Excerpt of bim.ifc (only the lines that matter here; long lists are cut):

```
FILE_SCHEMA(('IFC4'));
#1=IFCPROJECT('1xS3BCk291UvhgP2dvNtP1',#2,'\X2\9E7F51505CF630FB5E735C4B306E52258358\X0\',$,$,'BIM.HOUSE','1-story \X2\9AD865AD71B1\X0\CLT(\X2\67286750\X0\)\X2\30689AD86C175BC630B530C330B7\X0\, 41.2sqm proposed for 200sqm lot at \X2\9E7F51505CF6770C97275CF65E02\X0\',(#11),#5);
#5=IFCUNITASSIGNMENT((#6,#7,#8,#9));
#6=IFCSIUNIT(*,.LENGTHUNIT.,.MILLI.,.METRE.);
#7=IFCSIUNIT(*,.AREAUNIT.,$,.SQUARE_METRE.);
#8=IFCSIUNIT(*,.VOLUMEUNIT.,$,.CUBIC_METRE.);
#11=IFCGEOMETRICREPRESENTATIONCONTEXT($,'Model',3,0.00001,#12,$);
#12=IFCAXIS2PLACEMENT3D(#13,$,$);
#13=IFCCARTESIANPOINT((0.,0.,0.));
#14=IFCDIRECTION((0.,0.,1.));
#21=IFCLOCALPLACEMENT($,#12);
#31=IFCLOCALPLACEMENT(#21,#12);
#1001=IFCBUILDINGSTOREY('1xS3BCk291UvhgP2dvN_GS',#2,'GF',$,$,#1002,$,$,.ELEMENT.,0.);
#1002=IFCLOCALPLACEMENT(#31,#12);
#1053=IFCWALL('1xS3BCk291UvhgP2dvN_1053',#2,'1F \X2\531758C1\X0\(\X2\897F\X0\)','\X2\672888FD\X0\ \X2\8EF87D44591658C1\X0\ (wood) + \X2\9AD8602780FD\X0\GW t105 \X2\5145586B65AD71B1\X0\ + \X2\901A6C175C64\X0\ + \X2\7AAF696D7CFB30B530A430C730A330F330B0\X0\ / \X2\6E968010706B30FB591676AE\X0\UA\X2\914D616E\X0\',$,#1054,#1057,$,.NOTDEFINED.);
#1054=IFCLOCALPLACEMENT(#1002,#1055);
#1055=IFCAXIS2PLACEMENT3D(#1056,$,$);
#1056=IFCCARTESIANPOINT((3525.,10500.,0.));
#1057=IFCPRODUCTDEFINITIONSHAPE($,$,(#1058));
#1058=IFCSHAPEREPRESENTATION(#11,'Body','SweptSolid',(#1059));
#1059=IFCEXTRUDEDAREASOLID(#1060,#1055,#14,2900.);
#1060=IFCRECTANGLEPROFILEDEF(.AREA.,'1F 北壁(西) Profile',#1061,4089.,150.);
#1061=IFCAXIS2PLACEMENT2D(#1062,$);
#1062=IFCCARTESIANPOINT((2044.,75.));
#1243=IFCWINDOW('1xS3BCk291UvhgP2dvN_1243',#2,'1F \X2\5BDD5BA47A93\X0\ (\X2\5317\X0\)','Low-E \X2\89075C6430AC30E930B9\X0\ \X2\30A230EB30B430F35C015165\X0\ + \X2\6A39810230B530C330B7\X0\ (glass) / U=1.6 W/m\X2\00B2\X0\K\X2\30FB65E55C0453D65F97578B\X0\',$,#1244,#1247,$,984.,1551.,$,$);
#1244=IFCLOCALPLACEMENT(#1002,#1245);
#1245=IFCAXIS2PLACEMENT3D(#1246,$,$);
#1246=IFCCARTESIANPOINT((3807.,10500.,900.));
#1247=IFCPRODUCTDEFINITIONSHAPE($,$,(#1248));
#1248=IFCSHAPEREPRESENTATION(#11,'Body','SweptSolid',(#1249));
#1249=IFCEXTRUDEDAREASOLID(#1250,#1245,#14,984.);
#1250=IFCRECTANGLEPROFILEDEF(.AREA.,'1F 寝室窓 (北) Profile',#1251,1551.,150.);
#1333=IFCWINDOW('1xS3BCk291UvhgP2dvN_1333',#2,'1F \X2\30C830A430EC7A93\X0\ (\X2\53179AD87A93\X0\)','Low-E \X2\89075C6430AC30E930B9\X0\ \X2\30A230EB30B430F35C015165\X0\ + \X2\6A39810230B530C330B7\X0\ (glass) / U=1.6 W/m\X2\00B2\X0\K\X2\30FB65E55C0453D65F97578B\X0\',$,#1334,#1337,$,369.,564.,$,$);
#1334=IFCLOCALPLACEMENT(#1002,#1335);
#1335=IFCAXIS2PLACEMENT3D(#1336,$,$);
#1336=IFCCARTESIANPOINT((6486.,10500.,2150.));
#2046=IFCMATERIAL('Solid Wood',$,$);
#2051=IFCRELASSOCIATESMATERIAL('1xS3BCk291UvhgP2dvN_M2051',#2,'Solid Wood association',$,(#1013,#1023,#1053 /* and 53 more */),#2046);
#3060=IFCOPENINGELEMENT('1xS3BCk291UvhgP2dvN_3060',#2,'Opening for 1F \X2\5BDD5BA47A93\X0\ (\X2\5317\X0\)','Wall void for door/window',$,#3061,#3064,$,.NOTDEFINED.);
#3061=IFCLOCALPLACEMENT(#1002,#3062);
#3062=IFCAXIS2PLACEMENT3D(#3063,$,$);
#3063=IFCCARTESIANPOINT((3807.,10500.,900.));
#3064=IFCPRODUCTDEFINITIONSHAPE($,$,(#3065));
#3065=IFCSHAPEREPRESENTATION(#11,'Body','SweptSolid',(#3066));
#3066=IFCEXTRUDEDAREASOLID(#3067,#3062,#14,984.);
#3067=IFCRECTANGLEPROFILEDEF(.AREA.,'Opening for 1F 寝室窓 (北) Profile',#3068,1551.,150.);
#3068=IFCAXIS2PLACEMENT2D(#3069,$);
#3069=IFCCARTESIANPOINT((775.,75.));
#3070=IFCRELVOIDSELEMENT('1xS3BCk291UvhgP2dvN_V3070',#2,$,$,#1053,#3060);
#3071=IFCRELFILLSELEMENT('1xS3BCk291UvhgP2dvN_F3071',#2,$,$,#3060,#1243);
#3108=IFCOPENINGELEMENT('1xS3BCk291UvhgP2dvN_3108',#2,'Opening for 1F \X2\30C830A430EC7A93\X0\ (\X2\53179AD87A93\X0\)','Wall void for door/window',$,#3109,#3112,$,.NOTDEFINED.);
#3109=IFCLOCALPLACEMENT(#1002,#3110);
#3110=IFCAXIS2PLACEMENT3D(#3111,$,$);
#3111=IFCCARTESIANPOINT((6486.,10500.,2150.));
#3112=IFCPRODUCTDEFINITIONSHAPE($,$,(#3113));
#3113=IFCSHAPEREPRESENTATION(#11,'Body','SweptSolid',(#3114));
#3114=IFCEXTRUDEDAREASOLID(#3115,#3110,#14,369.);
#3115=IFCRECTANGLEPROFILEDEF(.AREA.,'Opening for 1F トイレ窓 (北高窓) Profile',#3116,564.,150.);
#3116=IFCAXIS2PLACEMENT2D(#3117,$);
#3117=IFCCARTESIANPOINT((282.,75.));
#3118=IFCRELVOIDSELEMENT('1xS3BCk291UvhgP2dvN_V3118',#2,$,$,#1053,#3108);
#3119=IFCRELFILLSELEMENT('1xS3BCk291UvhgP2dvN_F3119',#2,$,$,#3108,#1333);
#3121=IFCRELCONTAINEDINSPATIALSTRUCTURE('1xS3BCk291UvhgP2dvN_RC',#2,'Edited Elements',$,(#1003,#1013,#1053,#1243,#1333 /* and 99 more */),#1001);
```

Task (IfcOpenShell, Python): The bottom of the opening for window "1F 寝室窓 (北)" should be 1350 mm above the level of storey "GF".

```python
import numpy as np
import ifcopenshell
import ifcopenshell.api.geometry
import ifcopenshell.geom
import ifcopenshell.util.element
import ifcopenshell.util.placement
import ifcopenshell.util.shape
import ifcopenshell.util.unit

model = ifcopenshell.open("bim.ifc")
unit_scale = ifcopenshell.util.unit.calculate_unit_scale(model)

window = model.by_guid("1xS3BCk291UvhgP2dvN_1243")
opening = window.FillsVoids[0].RelatingOpeningElement
storey = ifcopenshell.util.element.get_container(window, ifc_class="IfcBuildingStorey")
level = ifcopenshell.util.placement.get_local_placement(storey.ObjectPlacement)[2, 3]

# The opening's origin need not be at the sill, so measure its lowest point.
shape = ifcopenshell.geom.create_shape(ifcopenshell.geom.settings(), opening)
bottom = ifcopenshell.util.shape.get_shape_bottom_elevation(shape, shape.geometry) / unit_scale
dz = level + 1.35 / unit_scale - bottom

shift = np.array([0.0, 0.0, dz])
# The window is not placed relative to its opening, so move both.
for product in (opening, window):
    matrix = ifcopenshell.util.placement.get_local_placement(product.ObjectPlacement)
    matrix[:3, 3] += shift
    ifcopenshell.api.geometry.edit_object_placement(model, product=product, matrix=matrix, is_si=False)

print(f"moved by {dz * unit_scale:+.3f} m")

model.write("bim_edited.ifc")
```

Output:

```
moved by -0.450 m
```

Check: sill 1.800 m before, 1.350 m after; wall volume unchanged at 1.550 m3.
